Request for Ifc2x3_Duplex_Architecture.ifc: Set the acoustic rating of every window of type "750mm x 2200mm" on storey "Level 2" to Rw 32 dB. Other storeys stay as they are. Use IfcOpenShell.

First a look at what the model holds.

```python
import ifcopenshell
import ifcopenshell.util.element

model = ifcopenshell.open("Ifc2x3_Duplex_Architecture.ifc")
print(model.schema)
storey = next(s for s in model.by_type("IfcBuildingStorey") if s.Name == "Level 2")
windows = [e for e in ifcopenshell.util.element.get_decomposition(storey) if e.is_a("IfcWindow")]
seen = {}
for e in windows:
    element_type = ifcopenshell.util.element.get_type(e)
    key = (element_type.Name if element_type != e and element_type else None, ifcopenshell.util.element.get_pset(e, "Pset_WindowCommon", "AcousticRating"))
    seen[key] = seen.get(key, 0) + 1
for (name, value), count in sorted(seen.items(), key=str):
    print(count, "x", name, "|", value)
```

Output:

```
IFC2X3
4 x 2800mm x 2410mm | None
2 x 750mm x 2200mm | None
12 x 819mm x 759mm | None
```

```python
import ifcopenshell
import ifcopenshell.api.pset
import ifcopenshell.util.element

model = ifcopenshell.open("Ifc2x3_Duplex_Architecture.ifc")

storey = next(s for s in model.by_type("IfcBuildingStorey") if s.Name == "Level 2")
windows = [e for e in ifcopenshell.util.element.get_decomposition(storey) if e.is_a("IfcWindow")]

count = 0
for e in windows:
    element_type = ifcopenshell.util.element.get_type(e)
    if element_type in (None, e) or element_type.Name != "750mm x 2200mm":
        continue
    # add_pset returns the element's existing set when there is one.
    pset = ifcopenshell.api.pset.add_pset(model, product=e, name="Pset_WindowCommon")
    ifcopenshell.api.pset.edit_pset(model, pset=pset, properties={"AcousticRating": "Rw 32 dB"})
    count += 1

print(count, "windows updated")

model.write("Ifc2x3_Duplex_Architecture_rev.ifc")
```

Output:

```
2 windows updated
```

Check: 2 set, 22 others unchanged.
